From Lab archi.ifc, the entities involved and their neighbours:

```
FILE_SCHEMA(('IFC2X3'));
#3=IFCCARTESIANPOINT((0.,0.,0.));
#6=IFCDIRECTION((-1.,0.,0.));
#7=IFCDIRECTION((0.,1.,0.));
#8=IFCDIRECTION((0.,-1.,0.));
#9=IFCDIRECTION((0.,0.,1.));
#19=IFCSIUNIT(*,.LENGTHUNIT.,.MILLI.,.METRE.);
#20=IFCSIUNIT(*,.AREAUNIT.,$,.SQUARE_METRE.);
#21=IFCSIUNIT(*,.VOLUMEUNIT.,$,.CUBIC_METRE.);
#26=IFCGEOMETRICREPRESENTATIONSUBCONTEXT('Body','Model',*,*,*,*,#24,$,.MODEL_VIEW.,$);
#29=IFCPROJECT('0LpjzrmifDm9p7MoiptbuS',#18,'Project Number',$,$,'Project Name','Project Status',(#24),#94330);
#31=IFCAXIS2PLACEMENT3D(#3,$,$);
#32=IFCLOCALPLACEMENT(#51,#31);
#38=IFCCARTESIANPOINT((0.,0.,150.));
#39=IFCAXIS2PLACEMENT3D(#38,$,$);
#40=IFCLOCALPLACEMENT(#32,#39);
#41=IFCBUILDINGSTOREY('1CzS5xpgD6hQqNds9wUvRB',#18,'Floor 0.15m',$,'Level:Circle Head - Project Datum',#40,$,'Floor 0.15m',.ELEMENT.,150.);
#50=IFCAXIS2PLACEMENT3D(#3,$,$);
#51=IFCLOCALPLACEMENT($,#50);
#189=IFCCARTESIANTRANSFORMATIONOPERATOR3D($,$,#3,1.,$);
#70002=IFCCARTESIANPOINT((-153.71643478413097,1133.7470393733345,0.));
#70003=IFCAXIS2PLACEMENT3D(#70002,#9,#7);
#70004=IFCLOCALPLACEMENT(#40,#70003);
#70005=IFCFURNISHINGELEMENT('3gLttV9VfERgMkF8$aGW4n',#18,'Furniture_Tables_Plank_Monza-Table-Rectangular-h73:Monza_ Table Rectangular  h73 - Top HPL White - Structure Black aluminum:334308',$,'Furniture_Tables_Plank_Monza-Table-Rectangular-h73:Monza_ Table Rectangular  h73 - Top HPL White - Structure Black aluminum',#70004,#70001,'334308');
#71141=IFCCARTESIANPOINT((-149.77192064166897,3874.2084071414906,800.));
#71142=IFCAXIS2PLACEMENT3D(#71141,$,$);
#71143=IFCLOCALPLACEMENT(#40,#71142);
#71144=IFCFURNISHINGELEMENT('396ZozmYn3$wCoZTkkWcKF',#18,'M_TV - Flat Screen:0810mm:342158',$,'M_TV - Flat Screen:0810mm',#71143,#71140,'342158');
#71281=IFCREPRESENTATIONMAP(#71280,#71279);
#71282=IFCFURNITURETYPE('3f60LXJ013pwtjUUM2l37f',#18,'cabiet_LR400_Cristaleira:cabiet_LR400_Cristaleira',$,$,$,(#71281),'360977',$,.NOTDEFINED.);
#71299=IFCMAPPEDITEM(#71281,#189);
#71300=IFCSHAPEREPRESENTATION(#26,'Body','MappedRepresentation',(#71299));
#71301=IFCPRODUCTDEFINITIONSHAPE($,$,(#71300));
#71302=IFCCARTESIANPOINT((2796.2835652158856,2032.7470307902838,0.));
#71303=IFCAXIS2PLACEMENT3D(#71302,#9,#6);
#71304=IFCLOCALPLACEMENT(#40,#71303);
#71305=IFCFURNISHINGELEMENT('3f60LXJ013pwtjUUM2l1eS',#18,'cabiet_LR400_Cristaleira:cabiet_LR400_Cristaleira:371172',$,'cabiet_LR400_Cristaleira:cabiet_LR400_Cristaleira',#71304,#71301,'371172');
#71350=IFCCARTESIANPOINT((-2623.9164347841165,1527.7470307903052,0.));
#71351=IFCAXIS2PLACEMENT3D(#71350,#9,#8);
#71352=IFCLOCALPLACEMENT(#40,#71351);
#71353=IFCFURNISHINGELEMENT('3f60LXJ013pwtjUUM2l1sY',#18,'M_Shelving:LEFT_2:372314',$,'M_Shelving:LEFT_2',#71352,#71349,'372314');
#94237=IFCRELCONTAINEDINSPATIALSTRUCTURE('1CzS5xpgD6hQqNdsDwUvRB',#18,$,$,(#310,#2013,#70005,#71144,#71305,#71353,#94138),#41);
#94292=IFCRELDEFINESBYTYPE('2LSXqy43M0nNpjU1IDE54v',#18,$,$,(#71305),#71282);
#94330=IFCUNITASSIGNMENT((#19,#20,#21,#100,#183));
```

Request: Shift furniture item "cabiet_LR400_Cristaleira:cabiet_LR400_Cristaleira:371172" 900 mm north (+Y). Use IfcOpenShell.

```python
import ifcopenshell
import ifcopenshell.api.geometry
import ifcopenshell.util.placement

model = ifcopenshell.open("Lab archi.ifc")

item = model.by_id(71305)
matrix = ifcopenshell.util.placement.get_local_placement(item.ObjectPlacement)
matrix[1, 3] += 900.0
ifcopenshell.api.geometry.edit_object_placement(model, product=item, matrix=matrix, is_si=False)

print(ifcopenshell.util.placement.get_local_placement(item.ObjectPlacement).round(3) + 0.0)

model.write("Lab archi_updated.ifc")
```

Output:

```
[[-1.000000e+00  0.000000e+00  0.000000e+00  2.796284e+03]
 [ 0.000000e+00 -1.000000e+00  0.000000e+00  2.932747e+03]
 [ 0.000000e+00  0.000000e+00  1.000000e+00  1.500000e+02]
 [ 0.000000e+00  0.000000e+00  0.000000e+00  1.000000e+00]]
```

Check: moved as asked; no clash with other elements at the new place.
